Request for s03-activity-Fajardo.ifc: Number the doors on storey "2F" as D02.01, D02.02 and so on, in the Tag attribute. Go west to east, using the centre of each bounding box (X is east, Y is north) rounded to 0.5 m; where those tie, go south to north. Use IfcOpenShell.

First a look at what the model holds.

```python
import ifcopenshell
import ifcopenshell.util.element
import ifcopenshell.util.placement

model = ifcopenshell.open("s03-activity-Fajardo.ifc")
print(model.schema)
storey = next(s for s in model.by_type("IfcBuildingStorey") if s.Name == "2F")
doors = [e for e in ifcopenshell.util.element.get_decomposition(storey) if e.is_a("IfcDoor")]
for e in sorted(doors, key=lambda e: e.id()):
    origin = ifcopenshell.util.placement.get_local_placement(e.ObjectPlacement)[:3, 3]
    print(e.id(), e.Tag, e.Name, origin.round(2) + 0.0, sep=" | ")
```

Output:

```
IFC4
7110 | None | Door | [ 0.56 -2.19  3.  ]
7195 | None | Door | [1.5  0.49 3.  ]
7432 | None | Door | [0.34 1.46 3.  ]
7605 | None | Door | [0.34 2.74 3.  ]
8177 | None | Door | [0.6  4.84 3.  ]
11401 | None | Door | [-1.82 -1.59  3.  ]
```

```python
import ifcopenshell
import ifcopenshell.geom
import ifcopenshell.util.element
import ifcopenshell.util.shape

model = ifcopenshell.open("s03-activity-Fajardo.ifc")
settings = ifcopenshell.geom.settings()
settings.set("use-world-coords", True)


def centre(element):
    shape = ifcopenshell.geom.create_shape(settings, element)
    return ifcopenshell.util.shape.get_bbox_centroid(shape.geometry)


storey = next(s for s in model.by_type("IfcBuildingStorey") if s.Name == "2F")
doors = [e for e in ifcopenshell.util.element.get_decomposition(storey) if e.is_a("IfcDoor")]

# Insertion points can sit at a corner or the storey origin, so sort by the geometry (in metres).
centres = {e: centre(e) for e in doors}
doors.sort(key=lambda e: (round(centres[e][0] / 0.5), centres[e][1]))

for i, e in enumerate(doors, start=1):
    number = f"D02.{i:02d}"
    e.Tag = number
    print(e.id(), number)

model.write("s03-activity-Fajardo_rev.ifc")
```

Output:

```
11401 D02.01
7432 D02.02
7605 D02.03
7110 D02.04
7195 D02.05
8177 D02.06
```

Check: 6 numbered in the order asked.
